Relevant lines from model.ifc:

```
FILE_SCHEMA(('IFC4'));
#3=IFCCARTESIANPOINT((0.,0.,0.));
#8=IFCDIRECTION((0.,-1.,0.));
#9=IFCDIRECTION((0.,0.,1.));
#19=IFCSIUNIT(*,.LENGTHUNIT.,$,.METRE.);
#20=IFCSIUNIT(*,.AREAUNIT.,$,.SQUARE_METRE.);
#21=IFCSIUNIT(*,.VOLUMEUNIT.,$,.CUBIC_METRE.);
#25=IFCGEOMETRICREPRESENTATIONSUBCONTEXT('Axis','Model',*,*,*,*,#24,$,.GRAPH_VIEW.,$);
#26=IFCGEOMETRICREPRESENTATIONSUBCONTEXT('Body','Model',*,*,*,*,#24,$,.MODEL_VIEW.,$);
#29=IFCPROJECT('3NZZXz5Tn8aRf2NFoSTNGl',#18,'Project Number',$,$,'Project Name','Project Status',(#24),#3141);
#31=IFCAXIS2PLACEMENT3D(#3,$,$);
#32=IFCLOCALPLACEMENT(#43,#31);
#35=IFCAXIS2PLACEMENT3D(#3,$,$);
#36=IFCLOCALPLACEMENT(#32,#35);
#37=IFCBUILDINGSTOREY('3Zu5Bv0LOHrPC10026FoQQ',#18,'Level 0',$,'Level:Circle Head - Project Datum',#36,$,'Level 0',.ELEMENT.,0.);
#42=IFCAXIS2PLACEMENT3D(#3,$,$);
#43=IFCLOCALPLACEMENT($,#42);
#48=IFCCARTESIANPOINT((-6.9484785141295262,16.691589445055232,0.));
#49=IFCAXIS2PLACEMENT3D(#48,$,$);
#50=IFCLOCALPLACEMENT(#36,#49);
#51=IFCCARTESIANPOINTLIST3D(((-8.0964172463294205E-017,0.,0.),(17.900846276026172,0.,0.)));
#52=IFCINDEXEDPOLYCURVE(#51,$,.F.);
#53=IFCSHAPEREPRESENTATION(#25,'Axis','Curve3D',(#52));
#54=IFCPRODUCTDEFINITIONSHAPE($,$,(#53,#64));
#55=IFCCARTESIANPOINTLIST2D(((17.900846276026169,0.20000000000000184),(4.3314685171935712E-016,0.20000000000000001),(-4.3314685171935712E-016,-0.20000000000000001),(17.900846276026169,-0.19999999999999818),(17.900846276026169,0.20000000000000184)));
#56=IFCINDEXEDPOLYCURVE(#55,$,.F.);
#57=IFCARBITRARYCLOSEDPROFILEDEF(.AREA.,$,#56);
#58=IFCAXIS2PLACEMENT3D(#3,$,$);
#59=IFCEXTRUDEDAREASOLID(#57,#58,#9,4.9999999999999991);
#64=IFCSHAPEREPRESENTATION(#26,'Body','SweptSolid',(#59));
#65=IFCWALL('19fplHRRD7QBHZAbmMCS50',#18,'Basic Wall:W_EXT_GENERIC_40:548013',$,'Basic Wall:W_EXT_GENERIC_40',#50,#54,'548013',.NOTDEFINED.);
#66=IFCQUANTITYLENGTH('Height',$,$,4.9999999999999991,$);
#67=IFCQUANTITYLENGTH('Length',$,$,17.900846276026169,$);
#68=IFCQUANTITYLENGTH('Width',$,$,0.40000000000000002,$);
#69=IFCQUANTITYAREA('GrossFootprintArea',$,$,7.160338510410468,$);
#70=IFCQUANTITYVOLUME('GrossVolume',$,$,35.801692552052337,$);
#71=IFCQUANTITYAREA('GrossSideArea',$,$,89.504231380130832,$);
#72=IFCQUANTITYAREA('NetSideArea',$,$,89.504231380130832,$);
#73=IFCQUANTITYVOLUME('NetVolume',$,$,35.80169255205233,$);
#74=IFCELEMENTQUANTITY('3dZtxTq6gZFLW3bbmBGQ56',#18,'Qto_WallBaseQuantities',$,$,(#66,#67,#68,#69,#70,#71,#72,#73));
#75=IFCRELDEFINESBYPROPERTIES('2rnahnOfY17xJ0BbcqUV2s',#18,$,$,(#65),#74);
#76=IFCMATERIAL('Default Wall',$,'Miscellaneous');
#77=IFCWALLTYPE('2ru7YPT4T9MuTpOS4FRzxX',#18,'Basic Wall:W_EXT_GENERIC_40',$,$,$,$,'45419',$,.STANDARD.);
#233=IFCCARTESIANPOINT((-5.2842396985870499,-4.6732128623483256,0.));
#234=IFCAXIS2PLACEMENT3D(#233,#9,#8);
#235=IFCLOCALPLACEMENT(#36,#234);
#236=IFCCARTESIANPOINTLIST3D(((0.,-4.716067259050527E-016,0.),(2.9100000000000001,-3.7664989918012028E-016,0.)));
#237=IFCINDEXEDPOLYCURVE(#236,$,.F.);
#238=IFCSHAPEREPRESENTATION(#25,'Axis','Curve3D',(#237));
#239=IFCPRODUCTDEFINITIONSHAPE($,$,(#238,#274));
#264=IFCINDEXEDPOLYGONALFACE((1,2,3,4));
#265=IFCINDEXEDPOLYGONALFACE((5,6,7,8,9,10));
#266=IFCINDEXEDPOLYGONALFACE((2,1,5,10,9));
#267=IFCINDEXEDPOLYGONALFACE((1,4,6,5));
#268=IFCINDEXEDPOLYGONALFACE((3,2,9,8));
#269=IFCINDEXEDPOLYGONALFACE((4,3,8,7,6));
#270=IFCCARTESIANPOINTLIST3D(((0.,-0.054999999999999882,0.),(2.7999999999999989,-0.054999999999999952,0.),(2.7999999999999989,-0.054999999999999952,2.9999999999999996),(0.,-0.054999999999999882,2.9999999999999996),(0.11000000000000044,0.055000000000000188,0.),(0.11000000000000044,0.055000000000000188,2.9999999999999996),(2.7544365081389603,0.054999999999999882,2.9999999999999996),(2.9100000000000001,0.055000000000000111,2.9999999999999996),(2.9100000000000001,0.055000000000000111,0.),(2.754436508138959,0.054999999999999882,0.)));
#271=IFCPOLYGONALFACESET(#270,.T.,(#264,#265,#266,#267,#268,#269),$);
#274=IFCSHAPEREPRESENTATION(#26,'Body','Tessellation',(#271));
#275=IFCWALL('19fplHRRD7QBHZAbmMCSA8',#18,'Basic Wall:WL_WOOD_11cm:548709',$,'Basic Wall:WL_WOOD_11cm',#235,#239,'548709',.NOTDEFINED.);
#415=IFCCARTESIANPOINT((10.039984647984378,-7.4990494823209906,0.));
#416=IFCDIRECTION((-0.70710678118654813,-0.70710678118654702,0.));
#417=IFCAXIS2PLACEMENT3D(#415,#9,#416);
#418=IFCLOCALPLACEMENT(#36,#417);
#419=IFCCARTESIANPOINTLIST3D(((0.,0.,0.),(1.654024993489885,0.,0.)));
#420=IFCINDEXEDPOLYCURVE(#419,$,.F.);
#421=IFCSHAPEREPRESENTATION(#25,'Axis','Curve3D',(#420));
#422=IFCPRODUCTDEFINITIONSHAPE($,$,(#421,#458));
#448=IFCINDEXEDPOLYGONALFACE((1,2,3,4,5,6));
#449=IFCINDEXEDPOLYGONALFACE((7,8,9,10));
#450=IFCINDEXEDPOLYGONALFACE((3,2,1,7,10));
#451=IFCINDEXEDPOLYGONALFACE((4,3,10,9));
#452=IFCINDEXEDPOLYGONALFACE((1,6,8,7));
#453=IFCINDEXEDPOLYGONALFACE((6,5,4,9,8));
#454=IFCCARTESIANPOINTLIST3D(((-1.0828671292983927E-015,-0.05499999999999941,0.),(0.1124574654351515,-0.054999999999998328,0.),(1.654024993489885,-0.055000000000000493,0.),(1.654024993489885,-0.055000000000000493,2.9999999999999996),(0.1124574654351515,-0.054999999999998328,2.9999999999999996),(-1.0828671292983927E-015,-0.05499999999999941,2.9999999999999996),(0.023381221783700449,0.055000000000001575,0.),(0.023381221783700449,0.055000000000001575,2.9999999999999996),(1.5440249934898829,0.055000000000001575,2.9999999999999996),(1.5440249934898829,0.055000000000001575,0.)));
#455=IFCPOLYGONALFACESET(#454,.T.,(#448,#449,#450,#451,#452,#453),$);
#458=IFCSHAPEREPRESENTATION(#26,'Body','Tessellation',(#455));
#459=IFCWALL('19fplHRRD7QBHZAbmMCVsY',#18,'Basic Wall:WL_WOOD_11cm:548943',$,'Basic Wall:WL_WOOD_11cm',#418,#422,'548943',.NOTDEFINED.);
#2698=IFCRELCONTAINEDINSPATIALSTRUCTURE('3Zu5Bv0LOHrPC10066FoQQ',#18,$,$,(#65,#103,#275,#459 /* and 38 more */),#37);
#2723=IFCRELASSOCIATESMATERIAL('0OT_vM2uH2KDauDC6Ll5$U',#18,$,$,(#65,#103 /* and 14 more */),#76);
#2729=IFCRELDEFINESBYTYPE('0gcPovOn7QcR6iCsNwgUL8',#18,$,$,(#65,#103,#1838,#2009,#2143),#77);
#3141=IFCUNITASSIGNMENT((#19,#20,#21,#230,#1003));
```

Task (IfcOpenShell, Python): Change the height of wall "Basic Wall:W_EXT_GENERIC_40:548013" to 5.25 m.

```python
import ifcopenshell
import ifcopenshell.api.pset
import ifcopenshell.geom
import ifcopenshell.util.element
import ifcopenshell.util.representation
import ifcopenshell.util.shape
import ifcopenshell.util.unit

model = ifcopenshell.open("model.ifc")
unit_scale = ifcopenshell.util.unit.calculate_unit_scale(model)
area_scale = ifcopenshell.util.unit.calculate_unit_scale(model, "AREAUNIT")
volume_scale = ifcopenshell.util.unit.calculate_unit_scale(model, "VOLUMEUNIT")
settings = ifcopenshell.geom.settings()


def volume(element):
    """Net volume in cubic metres, openings subtracted."""
    shape = ifcopenshell.geom.create_shape(settings, element)
    return ifcopenshell.util.shape.get_volume(shape.geometry)


wall = model.by_guid("19fplHRRD7QBHZAbmMCS50")
before = volume(wall)

body = ifcopenshell.util.representation.get_representation(wall, "Model", "Body")
solid = body.Items[0]
old_height = solid.Depth
solid.Depth = 5.25 / unit_scale
after = volume(wall)
thickness = 0.4  # wall thickness in metres

# Update the stored height, areas and volumes.
qto = model.by_id(ifcopenshell.util.element.get_pset(wall, "Qto_WallBaseQuantities", should_inherit=False)["id"])
ifcopenshell.api.pset.edit_qto(model, qto=qto, properties={
    "Height": solid.Depth,
    "GrossVolume": ifcopenshell.util.element.get_pset(wall, "Qto_WallBaseQuantities", "GrossVolume") * solid.Depth / old_height,
    "GrossSideArea": ifcopenshell.util.element.get_pset(wall, "Qto_WallBaseQuantities", "GrossSideArea") * solid.Depth / old_height,
    "NetSideArea": after / thickness / area_scale,
    "NetVolume": after / volume_scale,
})

print(f"height {old_height:g} -> {solid.Depth:g}, volume {before:.3f} -> {after:.3f} m3")

model.write("model_updated.ifc")
```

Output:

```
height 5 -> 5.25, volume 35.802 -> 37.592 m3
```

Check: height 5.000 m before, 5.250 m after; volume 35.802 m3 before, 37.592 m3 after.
